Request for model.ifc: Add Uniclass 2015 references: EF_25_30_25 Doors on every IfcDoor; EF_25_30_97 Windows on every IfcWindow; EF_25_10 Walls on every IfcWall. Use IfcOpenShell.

First a look at what the model holds.

```python
import ifcopenshell

model = ifcopenshell.open("model.ifc")
print(model.schema)
print("classifications:", [c.Name for c in model.by_type("IfcClassification")])
for ifc_class in ("IfcDoor", "IfcRoof", "IfcStair", "IfcWall", "IfcWindow"):
    print(ifc_class, len(model.by_type(ifc_class)))
```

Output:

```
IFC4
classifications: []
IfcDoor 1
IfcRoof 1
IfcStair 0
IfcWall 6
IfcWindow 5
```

```python
import ifcopenshell
import ifcopenshell.api.classification

model = ifcopenshell.open("model.ifc")

system = ifcopenshell.api.classification.add_classification(model, classification="Uniclass 2015")

codes = {
    "IfcDoor": ("EF_25_30_25", "Doors"),
    "IfcWindow": ("EF_25_30_97", "Windows"),
    "IfcWall": ("EF_25_10", "Walls"),
}
for ifc_class, (code, name) in codes.items():
    products = model.by_type(ifc_class)
    ifcopenshell.api.classification.add_reference(
        model, products=products, classification=system, identification=code, name=name
    )
    print(code, len(products))

model.write("model_rev.ifc")
```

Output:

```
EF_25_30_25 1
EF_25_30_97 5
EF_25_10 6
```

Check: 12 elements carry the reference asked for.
